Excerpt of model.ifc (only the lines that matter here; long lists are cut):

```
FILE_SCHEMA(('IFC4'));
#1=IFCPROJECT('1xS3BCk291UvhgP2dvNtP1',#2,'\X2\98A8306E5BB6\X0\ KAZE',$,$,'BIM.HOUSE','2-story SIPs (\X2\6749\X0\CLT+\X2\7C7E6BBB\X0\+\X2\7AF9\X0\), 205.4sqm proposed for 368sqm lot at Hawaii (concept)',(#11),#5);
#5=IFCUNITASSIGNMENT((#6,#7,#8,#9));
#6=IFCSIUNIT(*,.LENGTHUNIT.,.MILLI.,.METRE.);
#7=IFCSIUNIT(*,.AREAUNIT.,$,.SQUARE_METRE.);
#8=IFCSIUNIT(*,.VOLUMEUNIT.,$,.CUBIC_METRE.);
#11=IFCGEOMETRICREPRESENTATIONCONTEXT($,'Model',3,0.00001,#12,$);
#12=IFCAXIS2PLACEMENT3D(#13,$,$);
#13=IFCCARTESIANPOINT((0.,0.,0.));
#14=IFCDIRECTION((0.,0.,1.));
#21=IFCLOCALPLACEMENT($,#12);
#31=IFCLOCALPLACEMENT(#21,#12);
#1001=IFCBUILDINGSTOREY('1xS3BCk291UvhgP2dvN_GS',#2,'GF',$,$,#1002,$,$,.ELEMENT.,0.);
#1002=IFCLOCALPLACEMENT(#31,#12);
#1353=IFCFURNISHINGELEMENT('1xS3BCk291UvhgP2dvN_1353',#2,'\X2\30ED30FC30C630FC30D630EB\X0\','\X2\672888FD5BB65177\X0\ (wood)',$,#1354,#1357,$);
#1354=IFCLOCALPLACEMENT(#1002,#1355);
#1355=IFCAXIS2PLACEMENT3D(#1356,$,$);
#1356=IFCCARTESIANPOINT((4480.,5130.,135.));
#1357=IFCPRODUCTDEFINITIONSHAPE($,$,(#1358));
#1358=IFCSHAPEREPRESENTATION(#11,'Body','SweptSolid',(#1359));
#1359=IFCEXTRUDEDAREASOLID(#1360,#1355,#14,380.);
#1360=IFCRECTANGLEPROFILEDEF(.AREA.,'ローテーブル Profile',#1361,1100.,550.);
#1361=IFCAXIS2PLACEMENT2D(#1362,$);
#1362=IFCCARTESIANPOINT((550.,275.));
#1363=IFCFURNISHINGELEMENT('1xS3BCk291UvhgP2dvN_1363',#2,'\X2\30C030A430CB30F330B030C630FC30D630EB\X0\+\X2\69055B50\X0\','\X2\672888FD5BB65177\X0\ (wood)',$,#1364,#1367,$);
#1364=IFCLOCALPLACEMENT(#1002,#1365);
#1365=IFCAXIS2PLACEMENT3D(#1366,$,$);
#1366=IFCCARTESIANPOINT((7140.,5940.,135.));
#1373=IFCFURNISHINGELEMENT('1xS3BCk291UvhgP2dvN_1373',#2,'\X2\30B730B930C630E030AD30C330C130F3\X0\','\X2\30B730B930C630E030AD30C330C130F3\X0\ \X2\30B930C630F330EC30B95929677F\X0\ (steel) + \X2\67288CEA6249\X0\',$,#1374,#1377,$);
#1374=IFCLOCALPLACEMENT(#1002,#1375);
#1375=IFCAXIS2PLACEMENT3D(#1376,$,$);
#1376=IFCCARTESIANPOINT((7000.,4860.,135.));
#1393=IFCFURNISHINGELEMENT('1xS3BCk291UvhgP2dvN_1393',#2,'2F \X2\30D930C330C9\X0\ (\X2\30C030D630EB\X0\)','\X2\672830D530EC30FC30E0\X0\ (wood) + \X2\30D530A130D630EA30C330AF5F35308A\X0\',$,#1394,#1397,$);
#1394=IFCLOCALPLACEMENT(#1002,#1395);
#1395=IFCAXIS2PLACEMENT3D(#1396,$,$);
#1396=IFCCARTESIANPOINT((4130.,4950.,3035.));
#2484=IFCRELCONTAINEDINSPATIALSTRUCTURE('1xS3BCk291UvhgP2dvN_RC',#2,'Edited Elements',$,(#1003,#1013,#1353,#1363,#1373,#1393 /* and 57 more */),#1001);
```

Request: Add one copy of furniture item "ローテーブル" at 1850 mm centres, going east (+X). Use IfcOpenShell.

```python
import numpy as np
import ifcopenshell
import ifcopenshell.api.geometry
import ifcopenshell.api.root
import ifcopenshell.util.element
import ifcopenshell.util.placement
import ifcopenshell.util.unit

model = ifcopenshell.open("model.ifc")
unit_scale = ifcopenshell.util.unit.calculate_unit_scale(model)


def reuse_history(source, copy):
    """copy_class also copies each property set's owner history, people and application; keep the originals."""
    for rel in copy.IsDefinedBy:
        if rel.is_a("IfcRelDefinesByProperties") and (history := rel.RelatingPropertyDefinition.OwnerHistory):
            rel.RelatingPropertyDefinition.OwnerHistory = source.OwnerHistory
            ifcopenshell.util.element.remove_deep2(model, history)


source = model.by_guid("1xS3BCk291UvhgP2dvN_1353")
base = ifcopenshell.util.placement.get_local_placement(source.ObjectPlacement)
step = np.array([1.0, 0.0, 0.0]) * 1.85 / unit_scale

for i in range(1, 2):
    copy = ifcopenshell.api.root.copy_class(model, product=source)
    copy.Representation = ifcopenshell.util.element.copy_deep(
        model, source.Representation, exclude=["IfcGeometricRepresentationContext", "IfcRepresentationMap"]
    )
    reuse_history(source, copy)
    matrix = base.copy()
    matrix[:3, 3] += i * step
    print("added at", matrix[:3, 3].round(3) + 0.0)
    ifcopenshell.api.geometry.edit_object_placement(model, product=copy, matrix=matrix, is_si=False)

model.write("model_edited.ifc")
```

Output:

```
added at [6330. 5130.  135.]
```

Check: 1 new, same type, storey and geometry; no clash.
